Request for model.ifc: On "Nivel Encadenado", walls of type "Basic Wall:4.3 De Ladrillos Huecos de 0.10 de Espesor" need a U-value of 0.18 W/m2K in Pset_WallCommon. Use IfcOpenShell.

First a look at what the model holds.

```python
import ifcopenshell
import ifcopenshell.util.element

model = ifcopenshell.open("model.ifc")
print(model.schema)
storey = next(s for s in model.by_type("IfcBuildingStorey") if s.Name == "Nivel Encadenado")
walls = [e for e in ifcopenshell.util.element.get_decomposition(storey) if e.is_a("IfcWall")]
seen = {}
for e in walls:
    element_type = ifcopenshell.util.element.get_type(e)
    key = (element_type.Name if element_type != e and element_type else None, ifcopenshell.util.element.get_pset(e, "Pset_WallCommon", "ThermalTransmittance"))
    seen[key] = seen.get(key, 0) + 1
for (name, value), count in sorted(seen.items(), key=str):
    print(count, "x", name, "|", value)
```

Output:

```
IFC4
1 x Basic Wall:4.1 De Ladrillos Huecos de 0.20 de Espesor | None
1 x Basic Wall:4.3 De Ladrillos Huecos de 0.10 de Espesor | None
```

```python
import ifcopenshell
import ifcopenshell.api.pset
import ifcopenshell.util.element

model = ifcopenshell.open("model.ifc")

storey = next(s for s in model.by_type("IfcBuildingStorey") if s.Name == "Nivel Encadenado")
walls = [e for e in ifcopenshell.util.element.get_decomposition(storey) if e.is_a("IfcWall")]

count = 0
for e in walls:
    element_type = ifcopenshell.util.element.get_type(e)
    if element_type in (None, e) or element_type.Name != "Basic Wall:4.3 De Ladrillos Huecos de 0.10 de Espesor":
        continue
    # add_pset returns the element's existing set when there is one.
    pset = ifcopenshell.api.pset.add_pset(model, product=e, name="Pset_WallCommon")
    ifcopenshell.api.pset.edit_pset(model, pset=pset, properties={"ThermalTransmittance": 0.18})
    count += 1

print(count, "walls updated")

model.write("model_updated.ifc")
```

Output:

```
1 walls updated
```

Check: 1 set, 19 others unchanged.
